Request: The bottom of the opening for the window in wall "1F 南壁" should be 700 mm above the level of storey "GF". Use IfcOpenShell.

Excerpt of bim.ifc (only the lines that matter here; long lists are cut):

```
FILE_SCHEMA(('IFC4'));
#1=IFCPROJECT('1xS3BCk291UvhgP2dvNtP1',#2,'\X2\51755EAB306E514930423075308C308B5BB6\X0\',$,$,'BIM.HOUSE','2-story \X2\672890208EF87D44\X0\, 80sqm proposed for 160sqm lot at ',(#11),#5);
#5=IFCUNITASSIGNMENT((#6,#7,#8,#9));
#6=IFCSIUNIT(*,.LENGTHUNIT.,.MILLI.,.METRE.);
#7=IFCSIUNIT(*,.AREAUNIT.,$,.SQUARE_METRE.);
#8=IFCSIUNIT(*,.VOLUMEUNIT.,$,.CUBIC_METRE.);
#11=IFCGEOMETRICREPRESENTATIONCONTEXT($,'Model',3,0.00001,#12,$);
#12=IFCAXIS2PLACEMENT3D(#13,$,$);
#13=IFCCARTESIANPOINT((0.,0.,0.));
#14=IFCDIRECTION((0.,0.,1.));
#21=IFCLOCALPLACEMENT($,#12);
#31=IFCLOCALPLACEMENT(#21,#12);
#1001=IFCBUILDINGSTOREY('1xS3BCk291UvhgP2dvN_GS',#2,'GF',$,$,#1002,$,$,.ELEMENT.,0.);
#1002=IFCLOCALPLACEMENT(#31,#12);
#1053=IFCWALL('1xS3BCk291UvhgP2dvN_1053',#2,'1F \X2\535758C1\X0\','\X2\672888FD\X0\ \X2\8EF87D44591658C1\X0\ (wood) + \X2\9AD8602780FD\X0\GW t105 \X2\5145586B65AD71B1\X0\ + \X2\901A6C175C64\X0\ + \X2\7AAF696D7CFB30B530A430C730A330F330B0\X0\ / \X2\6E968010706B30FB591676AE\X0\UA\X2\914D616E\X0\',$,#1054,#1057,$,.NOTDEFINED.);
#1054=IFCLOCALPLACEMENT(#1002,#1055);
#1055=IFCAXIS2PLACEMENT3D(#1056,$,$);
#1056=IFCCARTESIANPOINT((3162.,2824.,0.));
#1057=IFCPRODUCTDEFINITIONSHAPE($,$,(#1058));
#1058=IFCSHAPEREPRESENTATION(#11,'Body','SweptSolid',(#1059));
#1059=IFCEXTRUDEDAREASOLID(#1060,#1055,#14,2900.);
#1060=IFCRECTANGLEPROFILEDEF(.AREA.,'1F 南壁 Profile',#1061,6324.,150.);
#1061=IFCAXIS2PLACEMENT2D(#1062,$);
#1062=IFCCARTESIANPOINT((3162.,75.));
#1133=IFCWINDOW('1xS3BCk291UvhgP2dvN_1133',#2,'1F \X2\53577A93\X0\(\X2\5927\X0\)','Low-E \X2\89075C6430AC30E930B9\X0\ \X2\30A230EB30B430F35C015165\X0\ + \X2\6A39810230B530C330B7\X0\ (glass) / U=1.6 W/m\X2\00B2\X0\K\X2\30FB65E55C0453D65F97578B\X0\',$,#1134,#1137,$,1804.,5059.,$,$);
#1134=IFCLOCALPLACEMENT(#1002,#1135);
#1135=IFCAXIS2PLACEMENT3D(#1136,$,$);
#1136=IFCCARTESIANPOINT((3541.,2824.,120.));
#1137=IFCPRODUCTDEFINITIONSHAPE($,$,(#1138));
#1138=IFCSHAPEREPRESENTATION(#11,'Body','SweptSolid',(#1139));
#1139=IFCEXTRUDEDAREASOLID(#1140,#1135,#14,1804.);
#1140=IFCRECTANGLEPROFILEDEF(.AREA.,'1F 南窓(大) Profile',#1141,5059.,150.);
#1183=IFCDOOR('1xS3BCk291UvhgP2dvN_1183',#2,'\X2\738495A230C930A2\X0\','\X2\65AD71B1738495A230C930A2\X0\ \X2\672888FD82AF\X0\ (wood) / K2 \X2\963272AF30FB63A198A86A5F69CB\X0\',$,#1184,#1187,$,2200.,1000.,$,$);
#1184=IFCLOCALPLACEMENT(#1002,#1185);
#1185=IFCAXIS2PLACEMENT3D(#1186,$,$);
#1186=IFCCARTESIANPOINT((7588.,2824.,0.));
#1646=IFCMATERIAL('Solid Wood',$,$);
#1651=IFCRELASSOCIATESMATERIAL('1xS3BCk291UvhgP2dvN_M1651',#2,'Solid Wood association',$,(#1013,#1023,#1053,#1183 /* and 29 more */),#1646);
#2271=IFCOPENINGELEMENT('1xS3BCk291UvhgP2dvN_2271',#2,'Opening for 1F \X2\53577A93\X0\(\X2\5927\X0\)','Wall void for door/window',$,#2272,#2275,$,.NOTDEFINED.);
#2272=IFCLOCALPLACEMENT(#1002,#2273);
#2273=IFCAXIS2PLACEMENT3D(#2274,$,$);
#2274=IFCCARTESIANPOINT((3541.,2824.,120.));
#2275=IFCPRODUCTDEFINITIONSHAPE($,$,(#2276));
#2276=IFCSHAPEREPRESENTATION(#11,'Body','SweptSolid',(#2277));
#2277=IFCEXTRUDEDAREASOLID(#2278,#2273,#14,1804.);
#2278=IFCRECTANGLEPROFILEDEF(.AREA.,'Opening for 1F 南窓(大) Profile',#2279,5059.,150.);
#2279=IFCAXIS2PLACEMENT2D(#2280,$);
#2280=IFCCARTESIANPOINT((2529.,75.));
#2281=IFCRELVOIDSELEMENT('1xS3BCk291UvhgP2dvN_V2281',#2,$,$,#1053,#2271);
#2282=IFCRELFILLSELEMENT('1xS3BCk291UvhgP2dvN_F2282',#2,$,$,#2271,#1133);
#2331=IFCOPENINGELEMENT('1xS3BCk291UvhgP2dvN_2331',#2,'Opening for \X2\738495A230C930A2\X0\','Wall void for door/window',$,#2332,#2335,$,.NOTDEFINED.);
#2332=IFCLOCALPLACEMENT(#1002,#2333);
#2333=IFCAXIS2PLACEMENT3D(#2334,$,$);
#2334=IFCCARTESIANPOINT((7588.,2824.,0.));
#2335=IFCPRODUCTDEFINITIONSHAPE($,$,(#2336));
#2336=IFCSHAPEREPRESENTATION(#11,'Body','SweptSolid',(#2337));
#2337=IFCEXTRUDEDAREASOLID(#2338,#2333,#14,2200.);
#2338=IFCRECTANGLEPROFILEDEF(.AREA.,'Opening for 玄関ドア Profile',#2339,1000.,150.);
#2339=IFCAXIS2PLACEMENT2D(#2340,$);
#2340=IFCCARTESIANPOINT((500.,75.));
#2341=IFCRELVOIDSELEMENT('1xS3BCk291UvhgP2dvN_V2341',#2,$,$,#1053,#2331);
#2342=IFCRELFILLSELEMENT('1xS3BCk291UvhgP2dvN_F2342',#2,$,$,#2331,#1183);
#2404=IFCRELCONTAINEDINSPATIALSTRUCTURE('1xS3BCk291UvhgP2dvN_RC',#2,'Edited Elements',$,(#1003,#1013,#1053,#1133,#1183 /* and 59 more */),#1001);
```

```python
import numpy as np
import ifcopenshell
import ifcopenshell.api.geometry
import ifcopenshell.geom
import ifcopenshell.util.element
import ifcopenshell.util.placement
import ifcopenshell.util.shape
import ifcopenshell.util.unit

model = ifcopenshell.open("bim.ifc")
unit_scale = ifcopenshell.util.unit.calculate_unit_scale(model)

window = model.by_guid("1xS3BCk291UvhgP2dvN_1133")
opening = window.FillsVoids[0].RelatingOpeningElement
storey = ifcopenshell.util.element.get_container(window, ifc_class="IfcBuildingStorey")
level = ifcopenshell.util.placement.get_local_placement(storey.ObjectPlacement)[2, 3]

# The opening's origin need not be at the sill, so measure its lowest point.
shape = ifcopenshell.geom.create_shape(ifcopenshell.geom.settings(), opening)
bottom = ifcopenshell.util.shape.get_shape_bottom_elevation(shape, shape.geometry) / unit_scale
dz = level + 0.7 / unit_scale - bottom

shift = np.array([0.0, 0.0, dz])
# The window is not placed relative to its opening, so move both.
for product in (opening, window):
    matrix = ifcopenshell.util.placement.get_local_placement(product.ObjectPlacement)
    matrix[:3, 3] += shift
    ifcopenshell.api.geometry.edit_object_placement(model, product=product, matrix=matrix, is_si=False)

print(f"moved by {dz * unit_scale:+.3f} m")

model.write("bim_v2.ifc")
```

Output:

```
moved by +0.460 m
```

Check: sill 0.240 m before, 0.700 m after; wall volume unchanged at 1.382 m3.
